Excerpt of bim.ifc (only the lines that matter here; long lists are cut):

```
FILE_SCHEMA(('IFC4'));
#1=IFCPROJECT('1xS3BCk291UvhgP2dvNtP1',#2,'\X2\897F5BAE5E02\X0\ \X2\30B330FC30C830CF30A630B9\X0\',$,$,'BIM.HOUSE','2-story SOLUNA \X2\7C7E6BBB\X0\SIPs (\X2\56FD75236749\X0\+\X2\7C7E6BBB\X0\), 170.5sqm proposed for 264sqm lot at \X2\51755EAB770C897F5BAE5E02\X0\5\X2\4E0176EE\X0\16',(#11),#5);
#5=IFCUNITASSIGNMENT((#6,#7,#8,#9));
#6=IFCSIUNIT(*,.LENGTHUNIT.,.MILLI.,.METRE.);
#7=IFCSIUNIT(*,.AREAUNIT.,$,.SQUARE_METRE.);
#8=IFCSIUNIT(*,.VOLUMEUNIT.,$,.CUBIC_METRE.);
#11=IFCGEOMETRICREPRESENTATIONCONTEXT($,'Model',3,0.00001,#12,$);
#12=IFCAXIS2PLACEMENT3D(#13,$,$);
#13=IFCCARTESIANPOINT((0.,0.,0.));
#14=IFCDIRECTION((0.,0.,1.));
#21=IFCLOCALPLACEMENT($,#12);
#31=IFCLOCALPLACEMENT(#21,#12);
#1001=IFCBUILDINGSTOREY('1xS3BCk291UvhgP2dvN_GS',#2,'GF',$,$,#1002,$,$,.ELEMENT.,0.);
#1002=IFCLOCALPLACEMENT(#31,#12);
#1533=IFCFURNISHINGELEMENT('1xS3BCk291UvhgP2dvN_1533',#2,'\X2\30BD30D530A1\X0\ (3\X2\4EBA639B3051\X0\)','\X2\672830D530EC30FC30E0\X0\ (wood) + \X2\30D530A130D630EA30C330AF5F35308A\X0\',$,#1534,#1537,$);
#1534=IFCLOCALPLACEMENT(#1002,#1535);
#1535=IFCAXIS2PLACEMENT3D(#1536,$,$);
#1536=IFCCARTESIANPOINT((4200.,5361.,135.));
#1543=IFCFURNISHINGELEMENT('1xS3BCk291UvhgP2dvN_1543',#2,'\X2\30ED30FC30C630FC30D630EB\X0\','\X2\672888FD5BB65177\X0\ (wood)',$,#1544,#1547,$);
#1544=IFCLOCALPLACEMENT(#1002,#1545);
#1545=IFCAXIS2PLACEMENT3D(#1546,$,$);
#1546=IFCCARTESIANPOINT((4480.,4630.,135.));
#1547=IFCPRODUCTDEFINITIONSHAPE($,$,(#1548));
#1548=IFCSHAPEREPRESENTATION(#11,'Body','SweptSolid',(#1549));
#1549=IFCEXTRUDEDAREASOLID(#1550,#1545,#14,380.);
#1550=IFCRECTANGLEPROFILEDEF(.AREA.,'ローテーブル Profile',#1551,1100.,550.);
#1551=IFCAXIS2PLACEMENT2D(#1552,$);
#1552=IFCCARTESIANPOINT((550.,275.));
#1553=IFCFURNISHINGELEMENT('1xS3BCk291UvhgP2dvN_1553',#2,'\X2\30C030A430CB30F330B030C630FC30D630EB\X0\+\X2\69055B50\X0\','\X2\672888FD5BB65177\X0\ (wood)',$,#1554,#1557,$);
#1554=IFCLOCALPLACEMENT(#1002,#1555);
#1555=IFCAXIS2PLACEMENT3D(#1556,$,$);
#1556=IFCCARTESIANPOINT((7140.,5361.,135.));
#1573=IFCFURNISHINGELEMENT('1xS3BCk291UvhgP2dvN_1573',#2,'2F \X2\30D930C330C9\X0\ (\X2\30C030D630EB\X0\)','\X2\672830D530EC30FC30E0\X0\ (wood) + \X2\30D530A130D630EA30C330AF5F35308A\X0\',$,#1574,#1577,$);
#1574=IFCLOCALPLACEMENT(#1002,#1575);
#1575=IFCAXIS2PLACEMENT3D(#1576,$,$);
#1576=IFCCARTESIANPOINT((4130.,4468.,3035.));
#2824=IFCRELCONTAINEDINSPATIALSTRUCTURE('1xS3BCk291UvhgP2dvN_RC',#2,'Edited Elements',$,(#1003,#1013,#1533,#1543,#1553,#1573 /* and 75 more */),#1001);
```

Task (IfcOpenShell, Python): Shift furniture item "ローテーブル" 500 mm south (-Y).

```python
import ifcopenshell
import ifcopenshell.api.geometry
import ifcopenshell.util.placement
import ifcopenshell.util.unit

model = ifcopenshell.open("bim.ifc")
unit_scale = ifcopenshell.util.unit.calculate_unit_scale(model)

item = model.by_id(1543)
matrix = ifcopenshell.util.placement.get_local_placement(item.ObjectPlacement)
matrix[1, 3] -= 0.5 / unit_scale
ifcopenshell.api.geometry.edit_object_placement(model, product=item, matrix=matrix, is_si=False)

print(ifcopenshell.util.placement.get_local_placement(item.ObjectPlacement).round(3) + 0.0)

model.write("bim_edited.ifc")
```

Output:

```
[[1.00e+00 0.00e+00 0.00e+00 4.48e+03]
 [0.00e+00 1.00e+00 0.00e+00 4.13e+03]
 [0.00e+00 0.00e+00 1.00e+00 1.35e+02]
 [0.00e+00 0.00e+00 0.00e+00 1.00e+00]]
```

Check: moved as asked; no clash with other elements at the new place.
